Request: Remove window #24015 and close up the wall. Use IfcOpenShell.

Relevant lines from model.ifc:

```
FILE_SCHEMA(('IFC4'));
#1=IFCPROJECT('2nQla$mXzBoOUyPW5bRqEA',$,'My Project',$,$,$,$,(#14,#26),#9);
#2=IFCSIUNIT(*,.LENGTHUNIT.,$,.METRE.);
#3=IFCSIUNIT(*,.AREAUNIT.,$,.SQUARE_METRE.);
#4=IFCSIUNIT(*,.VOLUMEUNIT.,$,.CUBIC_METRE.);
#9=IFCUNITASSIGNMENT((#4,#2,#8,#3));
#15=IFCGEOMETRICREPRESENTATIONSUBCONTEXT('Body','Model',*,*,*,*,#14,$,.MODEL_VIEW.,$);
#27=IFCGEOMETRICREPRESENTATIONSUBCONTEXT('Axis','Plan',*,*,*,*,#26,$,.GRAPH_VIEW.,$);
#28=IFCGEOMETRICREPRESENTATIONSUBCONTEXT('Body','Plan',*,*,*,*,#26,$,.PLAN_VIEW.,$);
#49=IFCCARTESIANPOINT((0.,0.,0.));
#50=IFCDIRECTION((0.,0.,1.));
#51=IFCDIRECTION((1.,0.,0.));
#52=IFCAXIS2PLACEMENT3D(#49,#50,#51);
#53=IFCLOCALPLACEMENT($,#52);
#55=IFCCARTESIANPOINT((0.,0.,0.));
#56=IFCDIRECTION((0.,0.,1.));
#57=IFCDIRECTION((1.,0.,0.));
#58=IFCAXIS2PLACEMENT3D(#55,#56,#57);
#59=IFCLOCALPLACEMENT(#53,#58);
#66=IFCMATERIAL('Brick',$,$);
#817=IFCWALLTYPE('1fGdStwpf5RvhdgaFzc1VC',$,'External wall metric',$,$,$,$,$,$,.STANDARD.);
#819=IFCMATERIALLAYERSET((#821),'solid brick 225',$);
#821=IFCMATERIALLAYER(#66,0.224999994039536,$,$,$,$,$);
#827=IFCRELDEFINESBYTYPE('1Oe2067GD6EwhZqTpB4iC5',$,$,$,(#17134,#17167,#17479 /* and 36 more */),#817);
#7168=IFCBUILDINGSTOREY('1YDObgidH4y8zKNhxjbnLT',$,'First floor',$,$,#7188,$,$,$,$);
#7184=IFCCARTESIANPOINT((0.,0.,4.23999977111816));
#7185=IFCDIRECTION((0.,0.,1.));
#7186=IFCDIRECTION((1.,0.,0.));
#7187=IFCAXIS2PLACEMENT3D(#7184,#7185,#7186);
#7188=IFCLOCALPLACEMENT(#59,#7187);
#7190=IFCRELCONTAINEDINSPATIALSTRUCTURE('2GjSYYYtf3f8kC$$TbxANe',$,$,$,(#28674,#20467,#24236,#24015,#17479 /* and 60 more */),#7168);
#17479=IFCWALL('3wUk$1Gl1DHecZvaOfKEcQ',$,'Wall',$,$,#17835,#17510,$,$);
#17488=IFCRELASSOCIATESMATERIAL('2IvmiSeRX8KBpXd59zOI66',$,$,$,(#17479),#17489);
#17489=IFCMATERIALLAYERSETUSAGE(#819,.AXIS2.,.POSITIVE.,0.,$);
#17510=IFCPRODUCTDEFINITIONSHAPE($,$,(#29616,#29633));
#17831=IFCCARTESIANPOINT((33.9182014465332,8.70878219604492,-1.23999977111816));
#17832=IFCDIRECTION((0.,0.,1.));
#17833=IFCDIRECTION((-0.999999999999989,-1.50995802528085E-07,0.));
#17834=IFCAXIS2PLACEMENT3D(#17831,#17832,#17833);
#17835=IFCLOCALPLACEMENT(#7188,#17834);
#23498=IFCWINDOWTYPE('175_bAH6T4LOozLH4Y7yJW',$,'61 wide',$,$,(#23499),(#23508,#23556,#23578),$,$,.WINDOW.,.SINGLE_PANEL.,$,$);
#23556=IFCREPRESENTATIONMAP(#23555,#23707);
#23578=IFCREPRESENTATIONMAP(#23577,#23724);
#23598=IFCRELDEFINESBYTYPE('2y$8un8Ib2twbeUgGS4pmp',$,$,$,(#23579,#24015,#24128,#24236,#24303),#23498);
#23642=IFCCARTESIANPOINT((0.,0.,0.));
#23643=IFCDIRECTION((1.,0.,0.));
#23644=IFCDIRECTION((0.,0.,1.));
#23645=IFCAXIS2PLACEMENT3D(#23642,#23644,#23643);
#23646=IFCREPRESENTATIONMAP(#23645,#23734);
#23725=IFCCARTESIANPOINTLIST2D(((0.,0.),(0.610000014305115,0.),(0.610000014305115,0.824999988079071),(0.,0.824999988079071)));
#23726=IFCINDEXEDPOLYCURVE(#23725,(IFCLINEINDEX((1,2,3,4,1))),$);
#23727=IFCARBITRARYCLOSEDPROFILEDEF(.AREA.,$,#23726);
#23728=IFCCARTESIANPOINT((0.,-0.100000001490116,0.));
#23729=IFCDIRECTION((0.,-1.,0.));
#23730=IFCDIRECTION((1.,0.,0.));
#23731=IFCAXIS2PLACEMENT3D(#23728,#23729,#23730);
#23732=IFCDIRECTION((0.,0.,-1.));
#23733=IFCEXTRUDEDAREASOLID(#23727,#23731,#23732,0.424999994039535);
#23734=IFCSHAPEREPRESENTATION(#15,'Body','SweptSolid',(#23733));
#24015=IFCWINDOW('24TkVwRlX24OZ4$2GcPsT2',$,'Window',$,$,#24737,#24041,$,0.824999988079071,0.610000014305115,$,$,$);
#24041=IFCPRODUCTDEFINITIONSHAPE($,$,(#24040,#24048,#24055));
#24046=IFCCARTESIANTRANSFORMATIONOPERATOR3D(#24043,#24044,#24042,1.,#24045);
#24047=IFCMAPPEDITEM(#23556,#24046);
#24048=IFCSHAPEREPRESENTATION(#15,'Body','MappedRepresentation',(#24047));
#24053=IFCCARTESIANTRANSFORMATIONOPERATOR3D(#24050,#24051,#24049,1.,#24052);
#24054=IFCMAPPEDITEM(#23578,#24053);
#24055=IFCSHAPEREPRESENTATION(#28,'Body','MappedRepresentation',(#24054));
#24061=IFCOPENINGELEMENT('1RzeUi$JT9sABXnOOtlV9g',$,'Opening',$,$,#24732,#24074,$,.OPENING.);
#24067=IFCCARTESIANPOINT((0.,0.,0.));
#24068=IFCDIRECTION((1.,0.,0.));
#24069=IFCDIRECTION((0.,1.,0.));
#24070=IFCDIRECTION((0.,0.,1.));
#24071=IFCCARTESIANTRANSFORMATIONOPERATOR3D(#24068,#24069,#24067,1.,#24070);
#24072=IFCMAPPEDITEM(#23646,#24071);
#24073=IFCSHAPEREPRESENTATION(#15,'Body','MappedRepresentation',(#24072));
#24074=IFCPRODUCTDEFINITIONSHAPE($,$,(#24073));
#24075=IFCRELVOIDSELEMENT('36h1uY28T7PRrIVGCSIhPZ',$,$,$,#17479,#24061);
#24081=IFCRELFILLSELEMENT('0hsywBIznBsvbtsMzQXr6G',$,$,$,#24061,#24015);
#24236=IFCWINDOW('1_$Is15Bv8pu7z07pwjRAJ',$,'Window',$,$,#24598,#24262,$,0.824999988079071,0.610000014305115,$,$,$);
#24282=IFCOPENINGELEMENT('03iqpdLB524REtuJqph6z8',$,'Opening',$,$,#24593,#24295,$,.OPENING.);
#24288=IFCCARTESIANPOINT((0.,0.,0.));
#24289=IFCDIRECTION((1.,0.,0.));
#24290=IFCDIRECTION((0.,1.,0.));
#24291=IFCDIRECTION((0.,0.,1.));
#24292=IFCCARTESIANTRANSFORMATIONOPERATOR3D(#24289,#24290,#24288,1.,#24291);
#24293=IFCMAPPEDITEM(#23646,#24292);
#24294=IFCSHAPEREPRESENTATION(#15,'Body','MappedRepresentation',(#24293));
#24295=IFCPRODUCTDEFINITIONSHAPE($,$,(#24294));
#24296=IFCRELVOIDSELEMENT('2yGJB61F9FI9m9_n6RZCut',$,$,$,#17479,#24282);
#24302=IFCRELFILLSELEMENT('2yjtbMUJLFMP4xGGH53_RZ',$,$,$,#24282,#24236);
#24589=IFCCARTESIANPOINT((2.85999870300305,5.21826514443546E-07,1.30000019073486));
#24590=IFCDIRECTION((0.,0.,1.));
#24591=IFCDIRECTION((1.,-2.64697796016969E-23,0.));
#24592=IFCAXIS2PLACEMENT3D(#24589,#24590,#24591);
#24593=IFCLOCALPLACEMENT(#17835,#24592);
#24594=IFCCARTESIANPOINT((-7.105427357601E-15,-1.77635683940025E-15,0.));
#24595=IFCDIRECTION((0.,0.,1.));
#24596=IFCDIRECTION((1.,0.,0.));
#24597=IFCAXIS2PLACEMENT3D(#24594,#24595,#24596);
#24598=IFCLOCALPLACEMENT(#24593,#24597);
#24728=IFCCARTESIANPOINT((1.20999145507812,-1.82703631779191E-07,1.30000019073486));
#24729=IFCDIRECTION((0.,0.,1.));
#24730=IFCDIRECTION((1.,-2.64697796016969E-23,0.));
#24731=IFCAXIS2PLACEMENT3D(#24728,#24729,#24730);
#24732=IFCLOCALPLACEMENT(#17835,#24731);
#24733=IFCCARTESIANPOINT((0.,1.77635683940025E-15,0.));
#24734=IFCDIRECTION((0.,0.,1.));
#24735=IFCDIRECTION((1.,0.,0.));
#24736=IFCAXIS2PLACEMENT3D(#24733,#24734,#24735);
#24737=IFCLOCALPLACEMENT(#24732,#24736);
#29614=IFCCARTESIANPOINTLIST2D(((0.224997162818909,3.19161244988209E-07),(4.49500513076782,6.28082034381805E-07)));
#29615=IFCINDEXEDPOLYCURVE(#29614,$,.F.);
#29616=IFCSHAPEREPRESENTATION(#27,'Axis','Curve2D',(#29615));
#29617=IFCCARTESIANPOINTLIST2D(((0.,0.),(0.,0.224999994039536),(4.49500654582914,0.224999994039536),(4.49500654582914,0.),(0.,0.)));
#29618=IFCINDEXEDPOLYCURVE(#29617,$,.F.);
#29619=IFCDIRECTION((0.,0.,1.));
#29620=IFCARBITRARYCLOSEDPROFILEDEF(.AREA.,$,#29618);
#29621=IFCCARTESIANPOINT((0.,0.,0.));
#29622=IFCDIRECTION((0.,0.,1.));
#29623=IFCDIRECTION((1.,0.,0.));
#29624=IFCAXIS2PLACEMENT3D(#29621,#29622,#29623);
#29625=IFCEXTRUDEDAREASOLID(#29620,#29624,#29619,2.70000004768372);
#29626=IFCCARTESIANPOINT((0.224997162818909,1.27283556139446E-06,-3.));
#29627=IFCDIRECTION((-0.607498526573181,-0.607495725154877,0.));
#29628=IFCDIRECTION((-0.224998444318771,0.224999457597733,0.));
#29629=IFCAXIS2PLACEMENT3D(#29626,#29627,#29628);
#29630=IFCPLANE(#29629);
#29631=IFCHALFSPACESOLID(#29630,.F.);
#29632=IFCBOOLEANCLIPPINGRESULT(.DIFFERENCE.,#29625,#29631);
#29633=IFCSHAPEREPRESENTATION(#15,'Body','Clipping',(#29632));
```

```python
import ifcopenshell
import ifcopenshell.api.feature
import ifcopenshell.api.root
import ifcopenshell.geom
import ifcopenshell.util.shape

model = ifcopenshell.open("model.ifc")
settings = ifcopenshell.geom.settings()


def volume(element):
    """Net volume in cubic metres, openings subtracted."""
    shape = ifcopenshell.geom.create_shape(settings, element)
    return ifcopenshell.util.shape.get_volume(shape.geometry)


window = model.by_guid("24TkVwRlX24OZ4$2GcPsT2")
opening = window.FillsVoids[0].RelatingOpeningElement
wall = opening.VoidsElements[0].RelatingBuildingElement
before = volume(wall)

ifcopenshell.api.root.remove_product(model, product=window)
ifcopenshell.api.feature.remove_feature(model, feature=opening)

after = volume(wall)

print(f"wall volume {before:.3f} -> {after:.3f} m3")

model.write("model_rev.ifc")
```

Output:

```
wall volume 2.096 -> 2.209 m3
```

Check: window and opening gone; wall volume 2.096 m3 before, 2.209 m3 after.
